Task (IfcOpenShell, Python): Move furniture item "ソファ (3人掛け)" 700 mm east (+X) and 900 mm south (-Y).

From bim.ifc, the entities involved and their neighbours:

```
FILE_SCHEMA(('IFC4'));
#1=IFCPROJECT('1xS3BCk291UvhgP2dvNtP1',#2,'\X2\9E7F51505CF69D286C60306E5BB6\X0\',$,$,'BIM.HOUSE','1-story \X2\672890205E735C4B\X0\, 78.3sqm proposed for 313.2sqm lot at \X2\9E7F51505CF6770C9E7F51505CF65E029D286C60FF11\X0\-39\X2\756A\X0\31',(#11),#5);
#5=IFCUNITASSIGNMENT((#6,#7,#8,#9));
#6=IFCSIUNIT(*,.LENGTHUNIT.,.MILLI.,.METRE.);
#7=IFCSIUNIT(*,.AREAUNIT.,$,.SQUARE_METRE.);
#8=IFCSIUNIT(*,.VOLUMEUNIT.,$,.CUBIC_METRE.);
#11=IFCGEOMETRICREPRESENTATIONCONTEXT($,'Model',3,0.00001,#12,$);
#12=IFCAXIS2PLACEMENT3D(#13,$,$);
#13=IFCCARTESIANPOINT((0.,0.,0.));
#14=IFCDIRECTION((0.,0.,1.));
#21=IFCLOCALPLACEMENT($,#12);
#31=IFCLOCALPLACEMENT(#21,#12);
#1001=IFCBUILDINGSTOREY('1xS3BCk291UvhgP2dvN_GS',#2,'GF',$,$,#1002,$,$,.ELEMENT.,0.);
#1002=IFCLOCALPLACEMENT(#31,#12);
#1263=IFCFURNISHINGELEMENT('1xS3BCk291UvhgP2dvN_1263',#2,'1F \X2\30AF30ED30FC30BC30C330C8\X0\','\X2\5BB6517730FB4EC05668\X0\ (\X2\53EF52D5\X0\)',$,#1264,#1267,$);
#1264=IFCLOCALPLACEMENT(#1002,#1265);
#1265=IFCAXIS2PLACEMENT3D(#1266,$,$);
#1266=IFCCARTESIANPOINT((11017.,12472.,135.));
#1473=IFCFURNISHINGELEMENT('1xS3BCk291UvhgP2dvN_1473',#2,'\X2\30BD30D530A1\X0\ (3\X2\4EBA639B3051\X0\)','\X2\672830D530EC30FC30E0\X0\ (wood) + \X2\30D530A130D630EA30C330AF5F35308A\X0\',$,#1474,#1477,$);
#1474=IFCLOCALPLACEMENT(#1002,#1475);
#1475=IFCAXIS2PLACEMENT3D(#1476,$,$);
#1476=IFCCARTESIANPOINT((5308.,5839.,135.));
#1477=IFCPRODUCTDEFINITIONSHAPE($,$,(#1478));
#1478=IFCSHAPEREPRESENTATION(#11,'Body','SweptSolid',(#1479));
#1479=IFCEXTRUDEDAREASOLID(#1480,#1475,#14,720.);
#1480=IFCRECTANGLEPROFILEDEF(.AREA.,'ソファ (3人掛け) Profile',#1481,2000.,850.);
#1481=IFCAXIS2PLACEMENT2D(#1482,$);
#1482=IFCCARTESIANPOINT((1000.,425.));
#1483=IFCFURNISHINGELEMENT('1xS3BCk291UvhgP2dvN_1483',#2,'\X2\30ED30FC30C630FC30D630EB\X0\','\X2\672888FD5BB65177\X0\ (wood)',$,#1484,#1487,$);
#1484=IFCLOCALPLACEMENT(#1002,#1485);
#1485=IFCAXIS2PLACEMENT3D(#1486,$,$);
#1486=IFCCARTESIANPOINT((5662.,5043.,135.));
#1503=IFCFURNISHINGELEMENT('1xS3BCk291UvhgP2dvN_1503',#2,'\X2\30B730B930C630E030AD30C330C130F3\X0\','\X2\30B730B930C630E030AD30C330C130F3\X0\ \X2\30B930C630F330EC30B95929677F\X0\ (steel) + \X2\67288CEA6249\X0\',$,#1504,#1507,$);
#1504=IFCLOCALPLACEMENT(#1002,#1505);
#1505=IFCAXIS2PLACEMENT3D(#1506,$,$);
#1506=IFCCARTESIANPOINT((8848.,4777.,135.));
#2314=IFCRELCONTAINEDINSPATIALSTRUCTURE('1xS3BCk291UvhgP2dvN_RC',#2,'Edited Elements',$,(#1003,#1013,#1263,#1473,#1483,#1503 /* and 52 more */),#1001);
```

```python
import ifcopenshell
import ifcopenshell.api.geometry
import ifcopenshell.util.placement
import ifcopenshell.util.unit

model = ifcopenshell.open("bim.ifc")
unit_scale = ifcopenshell.util.unit.calculate_unit_scale(model)

item = model.by_guid("1xS3BCk291UvhgP2dvN_1473")
matrix = ifcopenshell.util.placement.get_local_placement(item.ObjectPlacement)
matrix[0, 3] += 0.7 / unit_scale
matrix[1, 3] -= 0.9 / unit_scale
ifcopenshell.api.geometry.edit_object_placement(model, product=item, matrix=matrix, is_si=False)

print(ifcopenshell.util.placement.get_local_placement(item.ObjectPlacement).round(3) + 0.0)

model.write("bim_v2.ifc")
```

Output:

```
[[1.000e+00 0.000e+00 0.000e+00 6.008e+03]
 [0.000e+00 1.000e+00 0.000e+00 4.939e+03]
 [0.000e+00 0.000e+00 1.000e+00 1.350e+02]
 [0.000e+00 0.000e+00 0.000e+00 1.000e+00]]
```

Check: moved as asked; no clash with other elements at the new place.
